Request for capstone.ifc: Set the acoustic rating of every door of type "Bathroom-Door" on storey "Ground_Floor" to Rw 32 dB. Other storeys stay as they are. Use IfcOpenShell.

First a look at what the model holds.

```python
import ifcopenshell
import ifcopenshell.util.element

model = ifcopenshell.open("capstone.ifc")
print(model.schema)
storey = next(s for s in model.by_type("IfcBuildingStorey") if s.Name == "Ground_Floor")
doors = [e for e in ifcopenshell.util.element.get_decomposition(storey) if e.is_a("IfcDoor")]
seen = {}
for e in doors:
    element_type = ifcopenshell.util.element.get_type(e)
    key = (element_type.Name if element_type != e and element_type else None, ifcopenshell.util.element.get_pset(e, "Pset_DoorCommon", "AcousticRating"))
    seen[key] = seen.get(key, 0) + 1
for (name, value), count in sorted(seen.items(), key=str):
    print(count, "x", name, "|", value)
```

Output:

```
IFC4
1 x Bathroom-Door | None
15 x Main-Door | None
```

```python
import ifcopenshell
import ifcopenshell.api.pset
import ifcopenshell.util.element

model = ifcopenshell.open("capstone.ifc")

storey = next(s for s in model.by_type("IfcBuildingStorey") if s.Name == "Ground_Floor")
doors = [e for e in ifcopenshell.util.element.get_decomposition(storey) if e.is_a("IfcDoor")]

count = 0
for e in doors:
    element_type = ifcopenshell.util.element.get_type(e)
    if element_type in (None, e) or element_type.Name != "Bathroom-Door":
        continue
    # add_pset returns the element's existing set when there is one.
    pset = ifcopenshell.api.pset.add_pset(model, product=e, name="Pset_DoorCommon")
    ifcopenshell.api.pset.edit_pset(model, pset=pset, properties={"AcousticRating": "Rw 32 dB"})
    count += 1

print(count, "doors updated")

model.write("capstone-out.ifc")
```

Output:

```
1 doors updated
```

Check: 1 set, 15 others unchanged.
